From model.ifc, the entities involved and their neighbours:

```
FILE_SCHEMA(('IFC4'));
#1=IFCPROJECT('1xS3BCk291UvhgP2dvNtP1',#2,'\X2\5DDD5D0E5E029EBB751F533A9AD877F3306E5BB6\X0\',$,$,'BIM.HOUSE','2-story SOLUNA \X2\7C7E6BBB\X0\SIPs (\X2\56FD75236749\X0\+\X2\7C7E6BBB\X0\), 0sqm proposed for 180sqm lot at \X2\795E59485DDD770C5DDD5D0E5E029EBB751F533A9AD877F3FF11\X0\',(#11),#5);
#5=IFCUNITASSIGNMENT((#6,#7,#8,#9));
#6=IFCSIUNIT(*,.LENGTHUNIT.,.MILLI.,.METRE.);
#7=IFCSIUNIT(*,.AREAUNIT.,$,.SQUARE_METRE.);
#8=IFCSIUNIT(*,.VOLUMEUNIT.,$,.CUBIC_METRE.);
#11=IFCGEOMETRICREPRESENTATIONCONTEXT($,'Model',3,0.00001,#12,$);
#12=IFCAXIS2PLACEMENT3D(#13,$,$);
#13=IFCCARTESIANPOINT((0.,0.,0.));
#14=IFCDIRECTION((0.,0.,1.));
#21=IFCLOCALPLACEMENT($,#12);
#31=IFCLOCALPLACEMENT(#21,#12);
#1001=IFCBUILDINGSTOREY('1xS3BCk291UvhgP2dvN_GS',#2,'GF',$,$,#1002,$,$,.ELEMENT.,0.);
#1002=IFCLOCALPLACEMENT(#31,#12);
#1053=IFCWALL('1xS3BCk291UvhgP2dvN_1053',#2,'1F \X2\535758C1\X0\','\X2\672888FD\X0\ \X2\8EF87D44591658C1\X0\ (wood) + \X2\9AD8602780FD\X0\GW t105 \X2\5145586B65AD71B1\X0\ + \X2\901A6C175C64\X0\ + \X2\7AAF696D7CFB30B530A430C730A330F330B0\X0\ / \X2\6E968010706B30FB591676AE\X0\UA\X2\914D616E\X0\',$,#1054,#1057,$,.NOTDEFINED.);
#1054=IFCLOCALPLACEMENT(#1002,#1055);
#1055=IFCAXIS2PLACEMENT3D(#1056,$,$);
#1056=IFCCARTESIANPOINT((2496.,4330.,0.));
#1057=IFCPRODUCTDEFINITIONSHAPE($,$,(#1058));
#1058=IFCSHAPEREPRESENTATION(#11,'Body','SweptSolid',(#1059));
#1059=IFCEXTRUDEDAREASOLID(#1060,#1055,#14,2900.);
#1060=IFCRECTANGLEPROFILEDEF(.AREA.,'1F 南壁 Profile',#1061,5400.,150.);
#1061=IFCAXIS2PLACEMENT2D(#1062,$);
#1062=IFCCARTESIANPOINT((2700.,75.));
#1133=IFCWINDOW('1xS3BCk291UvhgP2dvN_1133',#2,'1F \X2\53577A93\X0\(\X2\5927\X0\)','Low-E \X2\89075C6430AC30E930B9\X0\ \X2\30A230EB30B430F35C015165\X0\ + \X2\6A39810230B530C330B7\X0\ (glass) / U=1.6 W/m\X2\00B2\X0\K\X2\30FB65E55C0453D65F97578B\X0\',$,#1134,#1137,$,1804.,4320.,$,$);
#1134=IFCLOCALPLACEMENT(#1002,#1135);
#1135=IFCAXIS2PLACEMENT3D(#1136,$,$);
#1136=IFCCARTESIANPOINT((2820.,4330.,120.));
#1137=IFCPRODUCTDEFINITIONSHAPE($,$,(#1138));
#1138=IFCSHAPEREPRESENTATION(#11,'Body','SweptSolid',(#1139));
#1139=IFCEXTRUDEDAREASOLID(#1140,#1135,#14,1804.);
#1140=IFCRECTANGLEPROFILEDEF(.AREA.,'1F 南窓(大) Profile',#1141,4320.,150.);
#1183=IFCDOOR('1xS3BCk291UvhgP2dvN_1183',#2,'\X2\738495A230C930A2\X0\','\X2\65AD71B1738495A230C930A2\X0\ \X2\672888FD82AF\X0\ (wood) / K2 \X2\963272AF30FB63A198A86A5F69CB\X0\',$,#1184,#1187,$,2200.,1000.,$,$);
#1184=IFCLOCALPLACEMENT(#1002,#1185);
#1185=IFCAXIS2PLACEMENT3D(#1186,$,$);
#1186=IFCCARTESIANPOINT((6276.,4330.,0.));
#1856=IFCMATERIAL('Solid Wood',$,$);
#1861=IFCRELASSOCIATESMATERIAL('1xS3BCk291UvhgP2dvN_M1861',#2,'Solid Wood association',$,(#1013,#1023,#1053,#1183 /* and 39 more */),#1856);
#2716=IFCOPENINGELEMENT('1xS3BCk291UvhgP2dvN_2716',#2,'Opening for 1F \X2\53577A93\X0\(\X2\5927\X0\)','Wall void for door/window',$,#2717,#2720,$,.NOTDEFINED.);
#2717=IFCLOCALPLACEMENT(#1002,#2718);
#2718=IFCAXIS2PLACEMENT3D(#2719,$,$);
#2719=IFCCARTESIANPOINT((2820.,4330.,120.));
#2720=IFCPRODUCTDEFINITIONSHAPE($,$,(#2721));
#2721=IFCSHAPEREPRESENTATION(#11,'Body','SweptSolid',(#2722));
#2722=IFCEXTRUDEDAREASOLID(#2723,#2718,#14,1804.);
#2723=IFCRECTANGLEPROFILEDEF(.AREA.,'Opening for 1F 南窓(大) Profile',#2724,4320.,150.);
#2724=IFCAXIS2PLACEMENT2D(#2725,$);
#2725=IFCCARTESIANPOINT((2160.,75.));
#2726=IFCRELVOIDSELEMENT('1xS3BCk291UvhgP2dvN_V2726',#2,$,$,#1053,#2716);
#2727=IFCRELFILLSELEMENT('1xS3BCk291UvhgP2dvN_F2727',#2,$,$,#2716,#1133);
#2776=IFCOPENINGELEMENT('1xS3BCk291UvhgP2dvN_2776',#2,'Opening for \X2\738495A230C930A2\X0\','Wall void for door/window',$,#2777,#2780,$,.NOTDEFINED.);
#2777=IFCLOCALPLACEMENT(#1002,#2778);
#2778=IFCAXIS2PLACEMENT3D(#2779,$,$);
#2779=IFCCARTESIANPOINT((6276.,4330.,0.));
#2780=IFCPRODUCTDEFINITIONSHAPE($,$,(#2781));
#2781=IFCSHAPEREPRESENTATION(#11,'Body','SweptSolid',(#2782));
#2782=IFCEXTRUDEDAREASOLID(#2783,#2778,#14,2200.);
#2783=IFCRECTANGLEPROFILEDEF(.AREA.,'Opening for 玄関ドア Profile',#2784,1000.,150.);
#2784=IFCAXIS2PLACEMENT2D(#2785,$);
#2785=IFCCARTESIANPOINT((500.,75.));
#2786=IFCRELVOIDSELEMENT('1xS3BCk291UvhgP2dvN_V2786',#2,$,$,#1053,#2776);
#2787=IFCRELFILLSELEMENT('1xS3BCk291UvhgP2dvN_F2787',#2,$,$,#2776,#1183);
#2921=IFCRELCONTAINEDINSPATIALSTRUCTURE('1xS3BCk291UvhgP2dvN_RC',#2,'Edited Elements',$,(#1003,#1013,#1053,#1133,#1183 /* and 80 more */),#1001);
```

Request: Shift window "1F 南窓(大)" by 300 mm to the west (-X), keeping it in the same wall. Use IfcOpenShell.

```python
import ifcopenshell
import ifcopenshell.api.geometry
import ifcopenshell.util.placement
import ifcopenshell.util.unit

model = ifcopenshell.open("model.ifc")
unit_scale = ifcopenshell.util.unit.calculate_unit_scale(model)

window = model.by_guid("1xS3BCk291UvhgP2dvN_1133")
opening = window.FillsVoids[0].RelatingOpeningElement
wall = opening.VoidsElements[0].RelatingBuildingElement

wall_matrix = ifcopenshell.util.placement.get_local_placement(wall.ObjectPlacement)
shift = wall_matrix[:3, 0] * -0.3 / unit_scale
before = ifcopenshell.util.placement.get_local_placement(window.ObjectPlacement)[:3, 3].copy()

# The window is not placed relative to its opening, so move both.
for product in (opening, window):
    matrix = ifcopenshell.util.placement.get_local_placement(product.ObjectPlacement)
    matrix[:3, 3] += shift
    ifcopenshell.api.geometry.edit_object_placement(model, product=product, matrix=matrix, is_si=False)

after = ifcopenshell.util.placement.get_local_placement(window.ObjectPlacement)[:3, 3]
print("window moved by", (after - before).round(3) + 0.0)

model.write("model_v2.ifc")
```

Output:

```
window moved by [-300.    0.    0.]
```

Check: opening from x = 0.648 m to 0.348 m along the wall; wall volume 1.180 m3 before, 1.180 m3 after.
